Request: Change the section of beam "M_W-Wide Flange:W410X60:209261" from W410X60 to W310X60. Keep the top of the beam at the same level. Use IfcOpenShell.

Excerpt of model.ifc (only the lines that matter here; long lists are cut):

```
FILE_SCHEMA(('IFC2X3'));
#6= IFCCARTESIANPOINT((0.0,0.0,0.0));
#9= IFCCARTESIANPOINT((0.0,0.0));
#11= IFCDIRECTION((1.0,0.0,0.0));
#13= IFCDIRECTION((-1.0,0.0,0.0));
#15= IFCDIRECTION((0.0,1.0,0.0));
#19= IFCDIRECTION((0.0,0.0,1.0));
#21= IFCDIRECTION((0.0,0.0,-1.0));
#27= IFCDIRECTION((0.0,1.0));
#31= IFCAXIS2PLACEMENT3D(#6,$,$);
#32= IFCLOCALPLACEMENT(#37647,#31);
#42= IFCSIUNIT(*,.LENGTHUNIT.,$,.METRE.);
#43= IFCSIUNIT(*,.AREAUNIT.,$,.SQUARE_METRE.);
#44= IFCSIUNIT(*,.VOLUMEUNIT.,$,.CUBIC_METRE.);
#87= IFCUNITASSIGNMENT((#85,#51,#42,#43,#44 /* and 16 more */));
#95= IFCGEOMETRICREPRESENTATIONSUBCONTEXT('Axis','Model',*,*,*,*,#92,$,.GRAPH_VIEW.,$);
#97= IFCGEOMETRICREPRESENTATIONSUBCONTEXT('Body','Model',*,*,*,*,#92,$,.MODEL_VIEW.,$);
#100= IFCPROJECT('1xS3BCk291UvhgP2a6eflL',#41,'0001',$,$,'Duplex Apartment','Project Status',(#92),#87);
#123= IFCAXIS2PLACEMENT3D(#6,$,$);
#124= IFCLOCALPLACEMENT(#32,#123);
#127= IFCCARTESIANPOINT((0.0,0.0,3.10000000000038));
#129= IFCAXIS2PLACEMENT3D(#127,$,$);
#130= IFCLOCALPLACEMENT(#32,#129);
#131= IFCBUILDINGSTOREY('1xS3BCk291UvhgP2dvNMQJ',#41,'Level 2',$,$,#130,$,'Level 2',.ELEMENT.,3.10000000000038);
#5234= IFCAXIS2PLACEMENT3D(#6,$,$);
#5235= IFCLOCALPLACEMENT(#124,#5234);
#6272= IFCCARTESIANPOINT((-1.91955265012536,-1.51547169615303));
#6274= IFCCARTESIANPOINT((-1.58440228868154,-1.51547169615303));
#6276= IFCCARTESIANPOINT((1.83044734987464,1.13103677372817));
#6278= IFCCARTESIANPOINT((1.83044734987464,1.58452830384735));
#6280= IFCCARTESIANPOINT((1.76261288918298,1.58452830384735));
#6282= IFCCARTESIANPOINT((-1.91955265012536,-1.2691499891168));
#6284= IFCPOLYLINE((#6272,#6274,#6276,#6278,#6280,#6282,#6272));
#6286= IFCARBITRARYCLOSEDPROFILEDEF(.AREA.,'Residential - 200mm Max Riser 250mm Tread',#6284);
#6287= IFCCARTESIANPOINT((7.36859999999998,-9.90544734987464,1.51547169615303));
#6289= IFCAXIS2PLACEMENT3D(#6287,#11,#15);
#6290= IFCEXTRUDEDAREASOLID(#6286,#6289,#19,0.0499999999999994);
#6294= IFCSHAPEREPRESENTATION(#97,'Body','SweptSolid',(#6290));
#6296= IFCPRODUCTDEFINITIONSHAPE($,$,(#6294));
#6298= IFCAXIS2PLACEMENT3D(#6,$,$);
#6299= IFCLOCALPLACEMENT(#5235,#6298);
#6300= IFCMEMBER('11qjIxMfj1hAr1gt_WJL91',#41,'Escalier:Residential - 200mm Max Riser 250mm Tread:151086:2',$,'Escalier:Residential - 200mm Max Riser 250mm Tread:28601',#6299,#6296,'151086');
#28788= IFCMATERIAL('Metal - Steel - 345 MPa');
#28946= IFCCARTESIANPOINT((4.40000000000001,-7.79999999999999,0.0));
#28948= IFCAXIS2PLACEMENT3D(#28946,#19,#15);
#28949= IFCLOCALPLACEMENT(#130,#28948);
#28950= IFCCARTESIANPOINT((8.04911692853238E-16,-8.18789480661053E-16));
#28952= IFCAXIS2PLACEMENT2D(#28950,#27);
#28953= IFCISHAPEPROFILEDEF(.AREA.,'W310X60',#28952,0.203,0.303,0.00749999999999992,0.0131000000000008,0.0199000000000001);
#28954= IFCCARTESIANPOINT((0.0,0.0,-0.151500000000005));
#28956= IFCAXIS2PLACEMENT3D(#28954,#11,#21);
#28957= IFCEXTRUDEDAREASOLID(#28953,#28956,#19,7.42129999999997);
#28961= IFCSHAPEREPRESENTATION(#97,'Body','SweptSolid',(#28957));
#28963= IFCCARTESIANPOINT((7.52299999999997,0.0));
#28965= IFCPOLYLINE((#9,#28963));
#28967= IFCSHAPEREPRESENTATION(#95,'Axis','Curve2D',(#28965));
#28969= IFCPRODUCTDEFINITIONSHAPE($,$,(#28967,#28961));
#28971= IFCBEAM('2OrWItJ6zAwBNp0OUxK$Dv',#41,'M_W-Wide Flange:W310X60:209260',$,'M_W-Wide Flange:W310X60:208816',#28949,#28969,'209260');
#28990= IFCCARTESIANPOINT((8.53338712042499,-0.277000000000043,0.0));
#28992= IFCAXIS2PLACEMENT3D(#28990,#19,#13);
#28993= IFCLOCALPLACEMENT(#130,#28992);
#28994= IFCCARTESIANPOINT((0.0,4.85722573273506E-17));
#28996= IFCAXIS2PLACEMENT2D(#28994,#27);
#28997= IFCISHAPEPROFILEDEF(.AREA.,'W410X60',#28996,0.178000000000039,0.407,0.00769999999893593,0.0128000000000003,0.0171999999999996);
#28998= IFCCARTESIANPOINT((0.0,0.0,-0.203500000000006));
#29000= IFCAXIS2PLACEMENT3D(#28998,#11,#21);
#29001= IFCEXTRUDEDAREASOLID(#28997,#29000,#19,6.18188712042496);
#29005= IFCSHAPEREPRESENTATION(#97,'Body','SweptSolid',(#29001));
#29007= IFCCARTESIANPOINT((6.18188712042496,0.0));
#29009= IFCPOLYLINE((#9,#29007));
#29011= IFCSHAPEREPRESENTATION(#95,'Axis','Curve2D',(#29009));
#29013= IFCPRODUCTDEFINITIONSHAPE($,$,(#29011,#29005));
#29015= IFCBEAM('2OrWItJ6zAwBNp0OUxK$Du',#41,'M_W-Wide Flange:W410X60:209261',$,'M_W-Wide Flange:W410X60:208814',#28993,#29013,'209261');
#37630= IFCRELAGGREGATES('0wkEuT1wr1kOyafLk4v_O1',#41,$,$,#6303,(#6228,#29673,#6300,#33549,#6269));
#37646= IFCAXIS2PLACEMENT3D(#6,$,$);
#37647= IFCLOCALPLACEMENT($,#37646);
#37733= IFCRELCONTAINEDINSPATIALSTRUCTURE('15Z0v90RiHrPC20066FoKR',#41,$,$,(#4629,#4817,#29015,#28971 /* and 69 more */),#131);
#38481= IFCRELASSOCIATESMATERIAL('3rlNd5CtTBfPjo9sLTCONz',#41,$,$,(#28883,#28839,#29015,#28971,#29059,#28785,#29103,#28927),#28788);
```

```python
import ifcopenshell
import ifcopenshell.util.element
import ifcopenshell.util.representation

model = ifcopenshell.open("model.ifc")

member = model.by_id(29015)
source = next(p for p in model.by_type("IfcIShapeProfileDef") if p.ProfileName == "W310X60")

body = ifcopenshell.util.representation.get_representation(member, "Model", "Body")
solid = body.Items[0]
old_profile = solid.SweptArea

# Copy the section's sizes but keep this member's own profile position.
profile = ifcopenshell.util.element.copy(model, source)
# Profiles are centred, so shift by half the change in depth to hold the top.
shift = (old_profile.OverallDepth - profile.OverallDepth) / 2
x, y = old_profile.Position.Location.Coordinates
up = (-1.0, 0.0)  # upwards, in the solid's own plane
location = model.createIfcCartesianPoint((x + up[0] * shift, y + up[1] * shift))
profile.Position = model.createIfcAxis2Placement2D(location, old_profile.Position.RefDirection)
solid.SweptArea = profile
if not model.get_total_inverses(old_profile):
    ifcopenshell.util.element.remove_deep2(model, old_profile)
member.Name = member.Name.replace("W410X60", "W310X60")
member.ObjectType = member.ObjectType.replace("W410X60", "W310X60")

print(solid.SweptArea)

model.write("model_v2.ifc")
```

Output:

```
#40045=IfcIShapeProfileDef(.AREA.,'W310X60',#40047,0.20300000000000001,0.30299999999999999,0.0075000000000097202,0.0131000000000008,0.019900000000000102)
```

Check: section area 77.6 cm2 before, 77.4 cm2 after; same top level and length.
